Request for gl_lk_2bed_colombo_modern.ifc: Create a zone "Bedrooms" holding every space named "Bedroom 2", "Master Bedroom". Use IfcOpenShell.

First a look at what the model holds.

```python
import ifcopenshell

model = ifcopenshell.open("gl_lk_2bed_colombo_modern.ifc")
print(model.schema)
seen = {}
for space in model.by_type("IfcSpace"):
    seen[space.LongName] = seen.get(space.LongName, 0) + 1
for name, count in sorted(seen.items(), key=str):
    print(count, "x", name)
print("zones:", [z.Name for z in model.by_type("IfcZone")][:20])
```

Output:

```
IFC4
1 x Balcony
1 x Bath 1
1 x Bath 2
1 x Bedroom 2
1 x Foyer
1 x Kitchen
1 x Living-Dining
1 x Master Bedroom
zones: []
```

```python
import ifcopenshell
import ifcopenshell.api.group
import ifcopenshell.api.root

model = ifcopenshell.open("gl_lk_2bed_colombo_modern.ifc")

names = {"Bedroom 2", "Master Bedroom"}
spaces = [s for s in model.by_type("IfcSpace") if s.LongName in names]

zone = ifcopenshell.api.root.create_entity(model, ifc_class="IfcZone", name="Bedrooms")
ifcopenshell.api.group.assign_group(model, products=spaces, group=zone)
print(len(spaces), "spaces in", zone.Name)

model.write("gl_lk_2bed_colombo_modern_edited.ifc")
```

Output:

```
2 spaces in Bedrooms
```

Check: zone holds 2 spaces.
